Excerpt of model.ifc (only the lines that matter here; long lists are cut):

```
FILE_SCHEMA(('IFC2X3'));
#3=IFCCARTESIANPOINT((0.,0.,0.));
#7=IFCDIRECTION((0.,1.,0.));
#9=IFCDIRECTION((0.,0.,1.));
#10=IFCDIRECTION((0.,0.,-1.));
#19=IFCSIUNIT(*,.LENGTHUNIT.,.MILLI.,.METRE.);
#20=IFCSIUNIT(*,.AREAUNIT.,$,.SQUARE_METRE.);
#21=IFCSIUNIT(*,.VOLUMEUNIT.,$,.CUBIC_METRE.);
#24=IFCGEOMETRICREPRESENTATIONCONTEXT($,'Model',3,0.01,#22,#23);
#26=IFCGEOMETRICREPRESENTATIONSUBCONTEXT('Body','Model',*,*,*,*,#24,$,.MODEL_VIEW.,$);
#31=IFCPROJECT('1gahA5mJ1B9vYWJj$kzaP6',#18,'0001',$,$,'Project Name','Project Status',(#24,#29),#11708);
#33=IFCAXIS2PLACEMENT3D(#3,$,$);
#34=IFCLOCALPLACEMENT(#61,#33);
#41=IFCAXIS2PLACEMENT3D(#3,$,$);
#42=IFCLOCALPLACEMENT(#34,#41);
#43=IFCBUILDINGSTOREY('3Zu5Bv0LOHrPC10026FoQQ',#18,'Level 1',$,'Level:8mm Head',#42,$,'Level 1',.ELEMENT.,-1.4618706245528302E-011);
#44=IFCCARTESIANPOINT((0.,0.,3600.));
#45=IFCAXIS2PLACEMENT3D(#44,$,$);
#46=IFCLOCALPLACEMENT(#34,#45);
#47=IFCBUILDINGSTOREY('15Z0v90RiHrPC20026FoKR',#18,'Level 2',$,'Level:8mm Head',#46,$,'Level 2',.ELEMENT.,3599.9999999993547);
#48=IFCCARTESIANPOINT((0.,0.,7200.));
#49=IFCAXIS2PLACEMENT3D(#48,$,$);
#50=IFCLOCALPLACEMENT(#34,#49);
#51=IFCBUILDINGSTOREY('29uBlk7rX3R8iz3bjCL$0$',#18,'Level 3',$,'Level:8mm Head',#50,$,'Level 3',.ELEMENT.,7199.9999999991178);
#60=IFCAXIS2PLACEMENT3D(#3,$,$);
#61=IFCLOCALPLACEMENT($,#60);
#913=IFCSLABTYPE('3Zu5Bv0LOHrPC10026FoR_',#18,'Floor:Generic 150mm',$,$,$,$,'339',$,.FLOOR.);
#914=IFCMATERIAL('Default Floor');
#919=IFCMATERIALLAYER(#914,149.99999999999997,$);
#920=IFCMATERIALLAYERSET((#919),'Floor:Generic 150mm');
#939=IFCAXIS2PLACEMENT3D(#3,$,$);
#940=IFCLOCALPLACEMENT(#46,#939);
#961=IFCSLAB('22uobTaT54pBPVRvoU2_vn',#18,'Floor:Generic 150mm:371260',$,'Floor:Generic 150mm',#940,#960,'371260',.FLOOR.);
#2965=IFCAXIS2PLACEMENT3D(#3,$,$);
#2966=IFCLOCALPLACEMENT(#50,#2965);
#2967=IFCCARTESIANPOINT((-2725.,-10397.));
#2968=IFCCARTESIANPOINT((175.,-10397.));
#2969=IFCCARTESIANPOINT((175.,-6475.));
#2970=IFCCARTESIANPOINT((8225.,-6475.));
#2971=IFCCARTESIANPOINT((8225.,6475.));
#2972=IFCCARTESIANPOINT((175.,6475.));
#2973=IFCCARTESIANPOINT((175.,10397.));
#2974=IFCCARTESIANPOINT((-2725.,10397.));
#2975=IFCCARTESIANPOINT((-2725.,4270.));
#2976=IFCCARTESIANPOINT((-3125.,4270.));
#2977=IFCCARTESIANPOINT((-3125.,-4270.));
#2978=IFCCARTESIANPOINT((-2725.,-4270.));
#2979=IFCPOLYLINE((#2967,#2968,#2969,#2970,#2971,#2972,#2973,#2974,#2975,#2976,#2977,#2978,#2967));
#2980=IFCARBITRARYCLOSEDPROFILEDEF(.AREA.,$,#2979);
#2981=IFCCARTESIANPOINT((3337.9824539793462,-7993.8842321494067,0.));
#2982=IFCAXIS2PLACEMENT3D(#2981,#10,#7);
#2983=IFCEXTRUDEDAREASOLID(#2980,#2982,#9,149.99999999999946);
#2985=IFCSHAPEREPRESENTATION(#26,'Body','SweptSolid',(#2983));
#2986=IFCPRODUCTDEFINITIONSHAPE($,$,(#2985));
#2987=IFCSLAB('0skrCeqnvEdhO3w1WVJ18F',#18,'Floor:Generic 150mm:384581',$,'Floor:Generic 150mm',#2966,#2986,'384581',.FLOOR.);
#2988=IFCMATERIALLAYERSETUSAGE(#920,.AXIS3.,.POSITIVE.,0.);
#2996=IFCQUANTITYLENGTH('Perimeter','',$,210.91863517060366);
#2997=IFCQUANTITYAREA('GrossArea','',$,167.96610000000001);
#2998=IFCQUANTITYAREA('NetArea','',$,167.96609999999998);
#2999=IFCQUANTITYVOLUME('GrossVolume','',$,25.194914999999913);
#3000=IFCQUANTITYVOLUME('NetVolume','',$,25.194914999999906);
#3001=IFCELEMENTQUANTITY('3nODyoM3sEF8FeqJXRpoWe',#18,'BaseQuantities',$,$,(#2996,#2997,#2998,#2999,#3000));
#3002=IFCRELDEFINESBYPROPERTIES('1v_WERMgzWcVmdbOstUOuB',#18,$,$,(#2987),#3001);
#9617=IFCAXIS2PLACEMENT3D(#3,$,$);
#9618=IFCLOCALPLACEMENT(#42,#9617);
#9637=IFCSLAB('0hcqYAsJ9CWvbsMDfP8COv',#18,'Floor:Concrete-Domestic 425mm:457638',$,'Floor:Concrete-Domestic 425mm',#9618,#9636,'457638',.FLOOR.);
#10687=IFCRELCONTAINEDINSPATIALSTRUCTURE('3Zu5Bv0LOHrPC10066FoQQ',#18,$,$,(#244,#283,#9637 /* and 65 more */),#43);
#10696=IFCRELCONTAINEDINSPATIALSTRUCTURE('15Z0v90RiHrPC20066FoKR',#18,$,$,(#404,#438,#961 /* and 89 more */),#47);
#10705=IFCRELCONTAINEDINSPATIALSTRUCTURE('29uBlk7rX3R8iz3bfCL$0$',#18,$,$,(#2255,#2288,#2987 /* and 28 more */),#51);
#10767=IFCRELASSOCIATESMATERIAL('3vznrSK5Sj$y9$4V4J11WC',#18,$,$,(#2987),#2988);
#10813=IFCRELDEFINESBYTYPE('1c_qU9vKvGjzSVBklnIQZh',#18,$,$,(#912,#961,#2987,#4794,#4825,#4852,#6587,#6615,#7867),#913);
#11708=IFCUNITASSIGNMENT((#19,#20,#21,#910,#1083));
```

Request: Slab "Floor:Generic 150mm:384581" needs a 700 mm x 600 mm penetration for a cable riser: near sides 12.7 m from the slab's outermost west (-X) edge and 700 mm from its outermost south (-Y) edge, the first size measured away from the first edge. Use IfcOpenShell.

```python
import numpy as np
import ifcopenshell
import ifcopenshell.api.feature
import ifcopenshell.api.geometry
import ifcopenshell.api.pset
import ifcopenshell.api.root
import ifcopenshell.geom
import ifcopenshell.util.element
import ifcopenshell.util.placement
import ifcopenshell.util.representation
import ifcopenshell.util.shape
import ifcopenshell.util.unit

model = ifcopenshell.open("model.ifc")
unit_scale = ifcopenshell.util.unit.calculate_unit_scale(model)
area_scale = ifcopenshell.util.unit.calculate_unit_scale(model, "AREAUNIT")
volume_scale = ifcopenshell.util.unit.calculate_unit_scale(model, "VOLUMEUNIT")
settings = ifcopenshell.geom.settings()


def volume(element):
    """Net volume in cubic metres, openings subtracted."""
    shape = ifcopenshell.geom.create_shape(settings, element)
    return ifcopenshell.util.shape.get_volume(shape.geometry)


slab = model.by_guid("0skrCeqnvEdhO3w1WVJ18F")
before = volume(slab)

# Extent in the slab's own axes, in metres. The edges named are its -X and -Y sides.
slab_shape = ifcopenshell.geom.create_shape(settings, slab)
vertices = ifcopenshell.util.shape.get_vertices(slab_shape.geometry)
x_min, y_min, bottom = vertices.min(axis=0)
top = vertices[:, 2].max()

opening = ifcopenshell.api.root.create_entity(model, ifc_class="IfcOpeningElement", name="Cable riser opening")
context = ifcopenshell.util.representation.get_context(model, "Model", "Body", "MODEL_VIEW")
width, depth = 0.7, 0.6
outline = [(0.0, 0.0), (width, 0.0), (width, depth), (0.0, depth), (0.0, 0.0)]
# Overshoot both faces by 50 mm so the cut is clean.
shape = ifcopenshell.api.geometry.add_slab_representation(
    model, context=context, depth=top - bottom + 0.1, polyline=outline
)
ifcopenshell.api.geometry.assign_representation(model, product=opening, representation=shape)

matrix = ifcopenshell.util.placement.get_local_placement(slab.ObjectPlacement)
matrix[:, 3] = matrix @ np.append(np.array([x_min + 12.7, y_min + 0.7, bottom - 0.05]) / unit_scale, 1.0)
ifcopenshell.api.geometry.edit_object_placement(model, product=opening, matrix=matrix, is_si=False)
ifcopenshell.api.feature.add_feature(model, feature=opening, element=slab)

after = volume(slab)

# Update the slab's stored quantities.
qto = model.by_id(ifcopenshell.util.element.get_pset(slab, "BaseQuantities", should_inherit=False)["id"])
ifcopenshell.api.pset.edit_qto(model, qto=qto, properties={
    "NetArea": after / (top - bottom) / area_scale,
    "NetVolume": after / volume_scale,
})

print(f"slab volume {before:.3f} -> {after:.3f} m3")

model.write("model_v2.ifc")
```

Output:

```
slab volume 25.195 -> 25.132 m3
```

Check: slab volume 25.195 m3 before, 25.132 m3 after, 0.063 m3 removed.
